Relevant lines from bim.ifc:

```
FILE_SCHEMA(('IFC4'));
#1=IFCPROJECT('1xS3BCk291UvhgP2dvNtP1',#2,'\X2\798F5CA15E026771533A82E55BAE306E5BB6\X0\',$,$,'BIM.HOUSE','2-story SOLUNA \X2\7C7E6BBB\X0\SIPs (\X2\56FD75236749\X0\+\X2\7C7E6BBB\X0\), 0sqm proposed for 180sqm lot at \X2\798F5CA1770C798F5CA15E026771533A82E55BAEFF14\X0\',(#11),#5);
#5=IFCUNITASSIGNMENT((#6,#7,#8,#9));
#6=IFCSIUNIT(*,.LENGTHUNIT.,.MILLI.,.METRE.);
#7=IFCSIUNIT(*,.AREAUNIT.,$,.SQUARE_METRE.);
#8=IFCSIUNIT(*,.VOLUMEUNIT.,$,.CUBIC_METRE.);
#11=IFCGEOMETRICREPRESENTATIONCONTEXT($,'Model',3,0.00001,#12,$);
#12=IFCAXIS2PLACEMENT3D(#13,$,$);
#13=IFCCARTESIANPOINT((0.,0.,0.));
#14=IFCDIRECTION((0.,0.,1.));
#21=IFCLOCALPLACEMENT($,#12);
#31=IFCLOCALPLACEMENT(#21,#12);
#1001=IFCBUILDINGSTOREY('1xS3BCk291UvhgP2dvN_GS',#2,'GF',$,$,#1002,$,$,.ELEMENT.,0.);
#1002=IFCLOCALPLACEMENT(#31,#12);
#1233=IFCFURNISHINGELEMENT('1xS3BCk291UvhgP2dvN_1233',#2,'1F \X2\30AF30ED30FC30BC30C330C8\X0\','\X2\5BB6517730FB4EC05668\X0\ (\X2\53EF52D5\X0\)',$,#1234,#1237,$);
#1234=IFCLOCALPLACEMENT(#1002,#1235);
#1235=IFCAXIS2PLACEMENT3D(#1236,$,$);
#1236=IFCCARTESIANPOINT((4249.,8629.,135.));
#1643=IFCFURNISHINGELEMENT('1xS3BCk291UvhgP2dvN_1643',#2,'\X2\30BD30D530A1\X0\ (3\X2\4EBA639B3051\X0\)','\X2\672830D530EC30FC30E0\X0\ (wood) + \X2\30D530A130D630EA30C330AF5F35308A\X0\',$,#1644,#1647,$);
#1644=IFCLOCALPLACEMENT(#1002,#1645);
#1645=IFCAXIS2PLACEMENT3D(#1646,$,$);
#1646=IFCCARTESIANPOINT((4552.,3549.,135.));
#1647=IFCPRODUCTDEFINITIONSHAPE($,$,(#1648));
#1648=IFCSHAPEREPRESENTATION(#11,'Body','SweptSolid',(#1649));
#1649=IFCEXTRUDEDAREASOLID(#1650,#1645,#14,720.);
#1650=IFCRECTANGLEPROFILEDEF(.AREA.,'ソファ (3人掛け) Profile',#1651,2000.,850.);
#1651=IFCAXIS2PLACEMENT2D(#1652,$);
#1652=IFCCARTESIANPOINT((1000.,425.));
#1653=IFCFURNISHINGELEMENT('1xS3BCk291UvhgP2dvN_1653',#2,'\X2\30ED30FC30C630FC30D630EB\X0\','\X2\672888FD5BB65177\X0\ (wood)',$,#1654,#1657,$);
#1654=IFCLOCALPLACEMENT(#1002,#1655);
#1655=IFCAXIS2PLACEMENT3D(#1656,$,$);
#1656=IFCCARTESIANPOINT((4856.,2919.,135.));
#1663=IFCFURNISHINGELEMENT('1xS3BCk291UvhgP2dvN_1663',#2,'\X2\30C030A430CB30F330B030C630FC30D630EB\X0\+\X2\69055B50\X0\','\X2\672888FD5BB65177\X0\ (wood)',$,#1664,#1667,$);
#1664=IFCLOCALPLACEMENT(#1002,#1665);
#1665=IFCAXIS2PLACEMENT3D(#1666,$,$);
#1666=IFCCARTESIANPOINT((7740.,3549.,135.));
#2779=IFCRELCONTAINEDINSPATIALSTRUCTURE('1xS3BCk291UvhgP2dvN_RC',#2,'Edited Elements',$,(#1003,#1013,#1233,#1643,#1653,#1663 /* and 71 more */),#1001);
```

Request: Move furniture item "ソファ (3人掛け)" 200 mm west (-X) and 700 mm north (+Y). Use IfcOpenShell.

```python
import ifcopenshell
import ifcopenshell.api.geometry
import ifcopenshell.util.placement
import ifcopenshell.util.unit

model = ifcopenshell.open("bim.ifc")
unit_scale = ifcopenshell.util.unit.calculate_unit_scale(model)

item = model.by_guid("1xS3BCk291UvhgP2dvN_1643")
matrix = ifcopenshell.util.placement.get_local_placement(item.ObjectPlacement)
matrix[0, 3] -= 0.2 / unit_scale
matrix[1, 3] += 0.7 / unit_scale
ifcopenshell.api.geometry.edit_object_placement(model, product=item, matrix=matrix, is_si=False)

print(ifcopenshell.util.placement.get_local_placement(item.ObjectPlacement).round(3) + 0.0)

model.write("bim-out.ifc")
```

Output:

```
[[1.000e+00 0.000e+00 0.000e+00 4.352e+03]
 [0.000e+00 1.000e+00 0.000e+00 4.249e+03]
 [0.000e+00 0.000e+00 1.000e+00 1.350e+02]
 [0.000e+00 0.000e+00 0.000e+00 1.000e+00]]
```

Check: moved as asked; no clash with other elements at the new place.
